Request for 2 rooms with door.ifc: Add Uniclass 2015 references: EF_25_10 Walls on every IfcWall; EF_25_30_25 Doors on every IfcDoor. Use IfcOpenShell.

First a look at what the model holds.

```python
import ifcopenshell

model = ifcopenshell.open("2 rooms with door.ifc")
print(model.schema)
print("classifications:", [c.Name for c in model.by_type("IfcClassification")])
for ifc_class in ("IfcDoor", "IfcRoof", "IfcStair", "IfcWall", "IfcWindow"):
    print(ifc_class, len(model.by_type(ifc_class)))
```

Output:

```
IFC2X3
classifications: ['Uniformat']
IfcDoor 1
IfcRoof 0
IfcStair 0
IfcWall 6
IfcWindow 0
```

```python
import ifcopenshell
import ifcopenshell.api.classification

model = ifcopenshell.open("2 rooms with door.ifc")

# IFC2X3 requires Source and Edition and has no link from the project to the system.
system = model.create_entity("IfcClassification", Source="NBS", Edition="2015", Name="Uniclass 2015")

codes = {
    "IfcWall": ("EF_25_10", "Walls"),
    "IfcDoor": ("EF_25_30_25", "Doors"),
}
for ifc_class, (code, name) in codes.items():
    products = model.by_type(ifc_class)
    ifcopenshell.api.classification.add_reference(
        model, products=products, classification=system, identification=code, name=name
    )
    print(code, len(products))

model.write("2 rooms with door_v2.ifc")
```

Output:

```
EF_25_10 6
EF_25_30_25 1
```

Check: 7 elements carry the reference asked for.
